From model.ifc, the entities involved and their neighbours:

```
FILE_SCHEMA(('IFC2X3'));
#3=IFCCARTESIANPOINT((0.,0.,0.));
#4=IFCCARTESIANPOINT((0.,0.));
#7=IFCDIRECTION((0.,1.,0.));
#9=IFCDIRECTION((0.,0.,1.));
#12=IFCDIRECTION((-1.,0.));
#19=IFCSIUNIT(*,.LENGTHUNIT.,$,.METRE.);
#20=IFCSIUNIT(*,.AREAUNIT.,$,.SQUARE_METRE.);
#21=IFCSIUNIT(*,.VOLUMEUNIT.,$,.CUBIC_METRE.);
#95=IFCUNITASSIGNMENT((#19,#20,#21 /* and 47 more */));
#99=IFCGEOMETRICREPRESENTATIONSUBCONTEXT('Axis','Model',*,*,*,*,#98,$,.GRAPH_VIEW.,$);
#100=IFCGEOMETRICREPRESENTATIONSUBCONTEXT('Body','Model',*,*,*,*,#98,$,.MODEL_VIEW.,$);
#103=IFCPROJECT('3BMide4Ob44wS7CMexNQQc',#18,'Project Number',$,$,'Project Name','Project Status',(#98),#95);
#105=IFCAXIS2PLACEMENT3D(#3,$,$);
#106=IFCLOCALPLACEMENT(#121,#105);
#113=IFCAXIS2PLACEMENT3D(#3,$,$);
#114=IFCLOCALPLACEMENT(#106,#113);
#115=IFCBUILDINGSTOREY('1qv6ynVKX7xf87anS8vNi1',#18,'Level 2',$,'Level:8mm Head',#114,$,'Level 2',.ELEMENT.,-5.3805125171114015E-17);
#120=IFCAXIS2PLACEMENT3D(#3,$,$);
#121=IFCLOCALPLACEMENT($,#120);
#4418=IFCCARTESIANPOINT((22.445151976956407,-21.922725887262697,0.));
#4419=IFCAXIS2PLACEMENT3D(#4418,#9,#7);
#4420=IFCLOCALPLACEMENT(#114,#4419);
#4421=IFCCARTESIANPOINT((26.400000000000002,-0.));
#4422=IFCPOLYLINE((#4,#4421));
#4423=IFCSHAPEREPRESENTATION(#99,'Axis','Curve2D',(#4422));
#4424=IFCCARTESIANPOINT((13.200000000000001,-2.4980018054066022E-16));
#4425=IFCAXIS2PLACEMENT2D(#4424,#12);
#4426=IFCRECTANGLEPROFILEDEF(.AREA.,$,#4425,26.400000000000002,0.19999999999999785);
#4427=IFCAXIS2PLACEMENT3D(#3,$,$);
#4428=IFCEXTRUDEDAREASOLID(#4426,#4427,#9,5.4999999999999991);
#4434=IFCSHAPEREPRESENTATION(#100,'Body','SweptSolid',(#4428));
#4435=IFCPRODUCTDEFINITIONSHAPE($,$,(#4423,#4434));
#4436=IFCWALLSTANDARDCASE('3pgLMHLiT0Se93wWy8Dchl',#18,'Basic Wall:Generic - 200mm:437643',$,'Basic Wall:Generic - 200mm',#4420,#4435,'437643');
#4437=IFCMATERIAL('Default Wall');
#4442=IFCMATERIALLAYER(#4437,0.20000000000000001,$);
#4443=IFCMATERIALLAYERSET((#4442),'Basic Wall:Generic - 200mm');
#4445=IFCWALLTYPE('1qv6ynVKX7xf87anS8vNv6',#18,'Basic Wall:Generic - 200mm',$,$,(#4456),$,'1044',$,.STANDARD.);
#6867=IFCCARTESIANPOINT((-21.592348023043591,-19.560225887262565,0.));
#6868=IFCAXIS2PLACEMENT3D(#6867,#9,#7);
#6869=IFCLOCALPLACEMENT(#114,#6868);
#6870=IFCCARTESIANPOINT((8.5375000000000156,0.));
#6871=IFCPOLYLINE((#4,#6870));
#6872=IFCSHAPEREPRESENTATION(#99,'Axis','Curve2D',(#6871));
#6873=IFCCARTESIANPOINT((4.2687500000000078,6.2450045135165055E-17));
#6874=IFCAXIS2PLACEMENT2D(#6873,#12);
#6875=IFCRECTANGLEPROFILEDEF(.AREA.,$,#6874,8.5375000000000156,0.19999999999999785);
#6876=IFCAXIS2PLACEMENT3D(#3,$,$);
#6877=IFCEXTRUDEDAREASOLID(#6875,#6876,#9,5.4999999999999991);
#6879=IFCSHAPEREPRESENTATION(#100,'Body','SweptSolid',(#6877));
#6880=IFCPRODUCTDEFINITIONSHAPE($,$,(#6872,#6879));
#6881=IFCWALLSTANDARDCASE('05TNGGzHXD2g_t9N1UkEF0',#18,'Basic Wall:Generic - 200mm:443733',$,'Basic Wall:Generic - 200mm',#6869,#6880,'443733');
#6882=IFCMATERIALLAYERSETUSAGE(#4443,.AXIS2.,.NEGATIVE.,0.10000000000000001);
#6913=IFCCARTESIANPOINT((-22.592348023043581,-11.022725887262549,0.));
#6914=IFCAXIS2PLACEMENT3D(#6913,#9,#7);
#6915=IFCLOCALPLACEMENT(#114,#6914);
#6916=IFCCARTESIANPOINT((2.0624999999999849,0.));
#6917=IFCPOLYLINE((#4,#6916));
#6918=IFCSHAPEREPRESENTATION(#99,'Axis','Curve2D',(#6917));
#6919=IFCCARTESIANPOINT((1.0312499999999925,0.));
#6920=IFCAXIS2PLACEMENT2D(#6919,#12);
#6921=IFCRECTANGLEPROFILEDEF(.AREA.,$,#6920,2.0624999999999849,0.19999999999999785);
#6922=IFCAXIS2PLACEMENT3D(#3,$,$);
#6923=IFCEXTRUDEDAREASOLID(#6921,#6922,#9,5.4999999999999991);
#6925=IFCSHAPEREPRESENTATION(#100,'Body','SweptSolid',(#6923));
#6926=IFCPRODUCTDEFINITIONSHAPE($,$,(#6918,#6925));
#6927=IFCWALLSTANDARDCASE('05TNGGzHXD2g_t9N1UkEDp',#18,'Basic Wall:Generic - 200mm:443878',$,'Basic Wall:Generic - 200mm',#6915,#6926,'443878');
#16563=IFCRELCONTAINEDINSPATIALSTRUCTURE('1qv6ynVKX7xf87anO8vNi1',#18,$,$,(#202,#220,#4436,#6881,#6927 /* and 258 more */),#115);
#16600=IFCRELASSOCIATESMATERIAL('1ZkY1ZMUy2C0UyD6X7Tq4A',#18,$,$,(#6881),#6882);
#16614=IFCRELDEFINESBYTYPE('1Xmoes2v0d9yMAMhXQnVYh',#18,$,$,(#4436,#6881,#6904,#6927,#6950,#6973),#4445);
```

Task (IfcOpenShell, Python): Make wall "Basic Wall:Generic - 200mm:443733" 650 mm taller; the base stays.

```python
import ifcopenshell
import ifcopenshell.geom
import ifcopenshell.util.representation
import ifcopenshell.util.shape

model = ifcopenshell.open("model.ifc")
settings = ifcopenshell.geom.settings()


def volume(element):
    """Net volume in cubic metres, openings subtracted."""
    shape = ifcopenshell.geom.create_shape(settings, element)
    return ifcopenshell.util.shape.get_volume(shape.geometry)


wall = model.by_guid("05TNGGzHXD2g_t9N1UkEF0")
before = volume(wall)

body = ifcopenshell.util.representation.get_representation(wall, "Model", "Body")
solid = body.Items[0]
old_height = solid.Depth
solid.Depth += 0.65
after = volume(wall)

print(f"height {old_height:g} -> {solid.Depth:g}, volume {before:.3f} -> {after:.3f} m3")

model.write("model_updated.ifc")
```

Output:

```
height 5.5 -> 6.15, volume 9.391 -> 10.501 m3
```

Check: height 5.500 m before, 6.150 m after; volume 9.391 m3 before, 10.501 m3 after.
